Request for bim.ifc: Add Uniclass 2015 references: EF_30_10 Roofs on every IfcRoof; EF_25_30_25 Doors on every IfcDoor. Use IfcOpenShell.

First a look at what the model holds.

```python
import ifcopenshell

model = ifcopenshell.open("bim.ifc")
print(model.schema)
print("classifications:", [c.Name for c in model.by_type("IfcClassification")])
for ifc_class in ("IfcDoor", "IfcRoof", "IfcStair", "IfcWall", "IfcWindow"):
    print(ifc_class, len(model.by_type(ifc_class)))
```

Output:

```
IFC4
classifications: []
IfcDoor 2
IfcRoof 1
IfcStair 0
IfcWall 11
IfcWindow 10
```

```python
import ifcopenshell
import ifcopenshell.api.classification

model = ifcopenshell.open("bim.ifc")

system = ifcopenshell.api.classification.add_classification(model, classification="Uniclass 2015")

codes = {
    "IfcRoof": ("EF_30_10", "Roofs"),
    "IfcDoor": ("EF_25_30_25", "Doors"),
}
for ifc_class, (code, name) in codes.items():
    products = model.by_type(ifc_class)
    ifcopenshell.api.classification.add_reference(
        model, products=products, classification=system, identification=code, name=name
    )
    print(code, len(products))

model.write("bim-out.ifc")
```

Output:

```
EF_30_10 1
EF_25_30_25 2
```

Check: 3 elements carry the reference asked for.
